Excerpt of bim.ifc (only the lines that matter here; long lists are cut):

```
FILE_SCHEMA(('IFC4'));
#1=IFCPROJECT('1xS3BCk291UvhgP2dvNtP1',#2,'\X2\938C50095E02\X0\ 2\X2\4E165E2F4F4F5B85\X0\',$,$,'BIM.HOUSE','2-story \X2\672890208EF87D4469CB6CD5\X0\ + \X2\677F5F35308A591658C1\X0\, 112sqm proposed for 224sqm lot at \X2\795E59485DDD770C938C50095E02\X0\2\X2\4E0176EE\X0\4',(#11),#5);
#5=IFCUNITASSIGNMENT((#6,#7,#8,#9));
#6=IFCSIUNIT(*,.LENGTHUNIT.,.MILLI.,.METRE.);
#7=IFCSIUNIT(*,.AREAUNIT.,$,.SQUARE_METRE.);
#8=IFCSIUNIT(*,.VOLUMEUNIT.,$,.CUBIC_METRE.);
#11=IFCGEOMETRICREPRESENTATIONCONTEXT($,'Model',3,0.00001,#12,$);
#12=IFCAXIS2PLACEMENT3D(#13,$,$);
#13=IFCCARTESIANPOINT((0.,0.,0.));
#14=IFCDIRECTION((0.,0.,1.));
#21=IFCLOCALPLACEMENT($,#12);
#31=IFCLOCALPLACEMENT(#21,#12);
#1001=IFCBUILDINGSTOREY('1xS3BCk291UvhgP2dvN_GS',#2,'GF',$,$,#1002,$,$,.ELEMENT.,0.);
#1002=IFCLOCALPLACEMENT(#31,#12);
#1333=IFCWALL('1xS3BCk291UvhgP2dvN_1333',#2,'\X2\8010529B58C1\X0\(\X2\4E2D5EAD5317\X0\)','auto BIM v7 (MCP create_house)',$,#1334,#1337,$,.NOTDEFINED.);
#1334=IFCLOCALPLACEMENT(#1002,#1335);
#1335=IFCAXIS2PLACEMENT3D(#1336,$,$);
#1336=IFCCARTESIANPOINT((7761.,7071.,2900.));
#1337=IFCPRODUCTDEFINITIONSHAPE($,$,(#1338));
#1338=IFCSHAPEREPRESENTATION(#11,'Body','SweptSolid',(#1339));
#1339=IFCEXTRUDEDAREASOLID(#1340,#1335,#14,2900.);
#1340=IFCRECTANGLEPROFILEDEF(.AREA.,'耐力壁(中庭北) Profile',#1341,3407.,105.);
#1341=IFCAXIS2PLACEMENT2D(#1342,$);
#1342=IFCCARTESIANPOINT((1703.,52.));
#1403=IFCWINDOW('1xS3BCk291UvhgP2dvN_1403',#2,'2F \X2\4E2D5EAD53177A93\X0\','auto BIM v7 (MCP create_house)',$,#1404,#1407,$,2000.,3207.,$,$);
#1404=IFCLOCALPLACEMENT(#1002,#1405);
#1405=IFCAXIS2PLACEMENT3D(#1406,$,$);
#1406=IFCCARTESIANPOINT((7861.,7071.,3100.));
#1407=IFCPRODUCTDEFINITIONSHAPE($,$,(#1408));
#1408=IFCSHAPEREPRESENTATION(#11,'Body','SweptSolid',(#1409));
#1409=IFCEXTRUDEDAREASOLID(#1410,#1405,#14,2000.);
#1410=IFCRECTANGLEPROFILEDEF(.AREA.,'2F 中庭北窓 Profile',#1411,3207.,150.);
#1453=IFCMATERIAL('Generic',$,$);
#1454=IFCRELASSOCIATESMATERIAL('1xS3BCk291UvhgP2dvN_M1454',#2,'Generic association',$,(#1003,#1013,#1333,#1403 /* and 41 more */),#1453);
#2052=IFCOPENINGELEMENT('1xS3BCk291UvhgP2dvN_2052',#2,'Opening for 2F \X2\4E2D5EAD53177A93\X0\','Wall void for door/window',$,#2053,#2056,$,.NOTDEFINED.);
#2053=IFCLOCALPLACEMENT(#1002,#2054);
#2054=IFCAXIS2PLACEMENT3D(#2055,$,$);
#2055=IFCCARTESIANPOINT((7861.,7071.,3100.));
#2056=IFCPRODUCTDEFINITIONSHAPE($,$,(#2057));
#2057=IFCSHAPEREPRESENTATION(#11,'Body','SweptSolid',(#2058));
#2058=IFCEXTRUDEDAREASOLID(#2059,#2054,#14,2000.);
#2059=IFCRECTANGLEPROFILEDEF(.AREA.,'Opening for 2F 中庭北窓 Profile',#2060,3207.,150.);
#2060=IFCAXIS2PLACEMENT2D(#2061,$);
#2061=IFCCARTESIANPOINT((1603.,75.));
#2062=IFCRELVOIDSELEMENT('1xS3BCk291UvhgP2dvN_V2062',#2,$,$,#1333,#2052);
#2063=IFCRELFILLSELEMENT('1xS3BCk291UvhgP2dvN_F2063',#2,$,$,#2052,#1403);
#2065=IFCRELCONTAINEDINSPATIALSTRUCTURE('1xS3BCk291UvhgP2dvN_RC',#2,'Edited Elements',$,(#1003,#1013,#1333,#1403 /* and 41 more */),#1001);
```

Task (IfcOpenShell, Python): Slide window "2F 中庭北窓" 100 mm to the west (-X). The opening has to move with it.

```python
import ifcopenshell
import ifcopenshell.api.geometry
import ifcopenshell.util.placement

model = ifcopenshell.open("bim.ifc")

window = model.by_guid("1xS3BCk291UvhgP2dvN_1403")
opening = window.FillsVoids[0].RelatingOpeningElement
wall = opening.VoidsElements[0].RelatingBuildingElement

wall_matrix = ifcopenshell.util.placement.get_local_placement(wall.ObjectPlacement)
shift = wall_matrix[:3, 0] * -100.0
before = ifcopenshell.util.placement.get_local_placement(window.ObjectPlacement)[:3, 3].copy()

# The window is not placed relative to its opening, so move both.
for product in (opening, window):
    matrix = ifcopenshell.util.placement.get_local_placement(product.ObjectPlacement)
    matrix[:3, 3] += shift
    ifcopenshell.api.geometry.edit_object_placement(model, product=product, matrix=matrix, is_si=False)

after = ifcopenshell.util.placement.get_local_placement(window.ObjectPlacement)[:3, 3]
print("window moved by", (after - before).round(3) + 0.0)

model.write("bim_updated.ifc")
```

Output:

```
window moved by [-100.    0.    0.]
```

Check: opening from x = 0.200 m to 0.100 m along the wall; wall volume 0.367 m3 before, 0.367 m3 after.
